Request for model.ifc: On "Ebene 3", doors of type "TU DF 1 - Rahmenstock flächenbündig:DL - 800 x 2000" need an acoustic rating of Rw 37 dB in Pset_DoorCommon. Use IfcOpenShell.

First a look at what the model holds.

```python
import ifcopenshell
import ifcopenshell.util.element

model = ifcopenshell.open("model.ifc")
print(model.schema)
storey = next(s for s in model.by_type("IfcBuildingStorey") if s.Name == "Ebene 3")
doors = [e for e in ifcopenshell.util.element.get_decomposition(storey) if e.is_a("IfcDoor")]
seen = {}
for e in doors:
    element_type = ifcopenshell.util.element.get_type(e)
    key = (element_type.Name if element_type != e and element_type else None, ifcopenshell.util.element.get_pset(e, "Pset_DoorCommon", "AcousticRating"))
    seen[key] = seen.get(key, 0) + 1
for (name, value), count in sorted(seen.items(), key=str):
    print(count, "x", name, "|", value)
```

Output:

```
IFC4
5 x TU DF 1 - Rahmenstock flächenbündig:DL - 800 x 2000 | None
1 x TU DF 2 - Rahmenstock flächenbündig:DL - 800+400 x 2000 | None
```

```python
import ifcopenshell
import ifcopenshell.api.pset
import ifcopenshell.util.element

model = ifcopenshell.open("model.ifc")

storey = next(s for s in model.by_type("IfcBuildingStorey") if s.Name == "Ebene 3")
doors = [e for e in ifcopenshell.util.element.get_decomposition(storey) if e.is_a("IfcDoor")]

count = 0
for e in doors:
    element_type = ifcopenshell.util.element.get_type(e)
    if element_type in (None, e) or element_type.Name != "TU DF 1 - Rahmenstock flächenbündig:DL - 800 x 2000":
        continue
    # add_pset returns the element's existing set when there is one.
    pset = ifcopenshell.api.pset.add_pset(model, product=e, name="Pset_DoorCommon")
    ifcopenshell.api.pset.edit_pset(model, pset=pset, properties={"AcousticRating": "Rw 37 dB"})
    count += 1

print(count, "doors updated")

model.write("model_edited.ifc")
```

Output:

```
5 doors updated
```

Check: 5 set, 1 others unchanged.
